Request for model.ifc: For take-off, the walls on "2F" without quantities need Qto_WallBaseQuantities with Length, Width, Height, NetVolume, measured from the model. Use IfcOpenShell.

First a look at what the model holds.

```python
import ifcopenshell
import ifcopenshell.util.element
import ifcopenshell.util.unit

model = ifcopenshell.open("model.ifc")
print(model.schema)
for unit_type in ("LENGTHUNIT", "AREAUNIT", "VOLUMEUNIT"):
    print(unit_type, ifcopenshell.util.unit.calculate_unit_scale(model, unit_type))
storey = next(s for s in model.by_type("IfcBuildingStorey") if s.Name == "2F")
walls = [e for e in ifcopenshell.util.element.get_decomposition(storey) if e.is_a("IfcWall")]
for e in sorted(walls, key=lambda e: e.id()):
    print(e.id(), e.is_a(), e.Name, list(ifcopenshell.util.element.get_psets(e, qtos_only=True)), sep=" | ")
```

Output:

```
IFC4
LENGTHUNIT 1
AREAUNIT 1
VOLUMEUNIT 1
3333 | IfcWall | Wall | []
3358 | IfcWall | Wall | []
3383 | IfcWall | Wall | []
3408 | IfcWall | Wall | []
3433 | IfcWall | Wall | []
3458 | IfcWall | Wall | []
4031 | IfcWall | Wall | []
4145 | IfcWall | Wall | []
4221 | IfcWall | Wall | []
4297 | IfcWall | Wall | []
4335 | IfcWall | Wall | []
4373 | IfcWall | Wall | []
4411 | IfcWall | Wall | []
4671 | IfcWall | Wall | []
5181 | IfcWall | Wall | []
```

```python
import ifcopenshell
import ifcopenshell.api.pset
import ifcopenshell.geom
import ifcopenshell.util.element
import ifcopenshell.util.shape
import ifcopenshell.util.unit

model = ifcopenshell.open("model.ifc")
unit_scale = ifcopenshell.util.unit.calculate_unit_scale(model)
volume_scale = ifcopenshell.util.unit.calculate_unit_scale(model, "VOLUMEUNIT")
settings = ifcopenshell.geom.settings()

storey = next(s for s in model.by_type("IfcBuildingStorey") if s.Name == "2F")
walls = [e for e in ifcopenshell.util.element.get_decomposition(storey) if e.is_a("IfcWall")]

for e in sorted(walls, key=lambda e: e.id()):
    if ifcopenshell.util.element.get_psets(e, qtos_only=True, should_inherit=False):
        continue
    # Geometry comes back in metres, in the element's own axes.
    shape = ifcopenshell.geom.create_shape(settings, e)
    values = {
        "Length": ifcopenshell.util.shape.get_x(shape.geometry) / unit_scale,
        "Width": ifcopenshell.util.shape.get_y(shape.geometry) / unit_scale,
        "Height": ifcopenshell.util.shape.get_z(shape.geometry) / unit_scale,
        "NetVolume": ifcopenshell.util.shape.get_volume(shape.geometry) / volume_scale,
    }
    qto = ifcopenshell.api.pset.add_qto(model, product=e, name="Qto_WallBaseQuantities")
    ifcopenshell.api.pset.edit_qto(model, qto=qto, properties=values)
    print(e.id(), {k: round(v, 3) for k, v in values.items()})

model.write("model_rev.ifc")
```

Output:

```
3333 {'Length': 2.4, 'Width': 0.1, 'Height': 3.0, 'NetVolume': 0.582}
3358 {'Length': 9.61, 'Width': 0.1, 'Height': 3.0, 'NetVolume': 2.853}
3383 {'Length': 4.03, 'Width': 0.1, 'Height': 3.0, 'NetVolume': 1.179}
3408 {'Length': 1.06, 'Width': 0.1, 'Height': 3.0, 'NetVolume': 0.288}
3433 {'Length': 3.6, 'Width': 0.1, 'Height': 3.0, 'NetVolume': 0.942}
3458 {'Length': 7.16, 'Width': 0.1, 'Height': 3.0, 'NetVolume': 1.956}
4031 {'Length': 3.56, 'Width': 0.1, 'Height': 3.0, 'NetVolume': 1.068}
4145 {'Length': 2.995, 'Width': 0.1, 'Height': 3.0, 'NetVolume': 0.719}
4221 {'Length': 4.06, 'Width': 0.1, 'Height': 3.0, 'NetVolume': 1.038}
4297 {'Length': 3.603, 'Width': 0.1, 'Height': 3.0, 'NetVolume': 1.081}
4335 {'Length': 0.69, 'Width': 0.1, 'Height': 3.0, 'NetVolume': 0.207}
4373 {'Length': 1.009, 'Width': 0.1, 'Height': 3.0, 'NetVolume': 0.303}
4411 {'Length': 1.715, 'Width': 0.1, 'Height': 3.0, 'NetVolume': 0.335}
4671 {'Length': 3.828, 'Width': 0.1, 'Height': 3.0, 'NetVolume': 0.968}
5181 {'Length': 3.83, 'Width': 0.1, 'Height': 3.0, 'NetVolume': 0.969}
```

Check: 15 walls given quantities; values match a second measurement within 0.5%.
